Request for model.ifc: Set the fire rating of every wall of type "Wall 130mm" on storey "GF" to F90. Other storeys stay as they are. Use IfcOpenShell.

First a look at what the model holds.

```python
import ifcopenshell
import ifcopenshell.util.element

model = ifcopenshell.open("model.ifc")
print(model.schema)
storey = next(s for s in model.by_type("IfcBuildingStorey") if s.Name == "GF")
walls = [e for e in ifcopenshell.util.element.get_decomposition(storey) if e.is_a("IfcWall")]
seen = {}
for e in walls:
    element_type = ifcopenshell.util.element.get_type(e)
    key = (element_type.Name if element_type != e and element_type else None, ifcopenshell.util.element.get_pset(e, "Pset_WallCommon", "FireRating"))
    seen[key] = seen.get(key, 0) + 1
for (name, value), count in sorted(seen.items(), key=str):
    print(count, "x", name, "|", value)
```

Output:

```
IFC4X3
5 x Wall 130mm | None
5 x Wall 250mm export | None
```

```python
import ifcopenshell
import ifcopenshell.api.pset
import ifcopenshell.util.element

model = ifcopenshell.open("model.ifc")

storey = next(s for s in model.by_type("IfcBuildingStorey") if s.Name == "GF")
walls = [e for e in ifcopenshell.util.element.get_decomposition(storey) if e.is_a("IfcWall")]

count = 0
for e in walls:
    element_type = ifcopenshell.util.element.get_type(e)
    if element_type in (None, e) or element_type.Name != "Wall 130mm":
        continue
    # add_pset returns the element's existing set when there is one.
    pset = ifcopenshell.api.pset.add_pset(model, product=e, name="Pset_WallCommon")
    ifcopenshell.api.pset.edit_pset(model, pset=pset, properties={"FireRating": "F90"})
    count += 1

print(count, "walls updated")

model.write("model_rev.ifc")
```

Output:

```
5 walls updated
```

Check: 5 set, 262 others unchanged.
